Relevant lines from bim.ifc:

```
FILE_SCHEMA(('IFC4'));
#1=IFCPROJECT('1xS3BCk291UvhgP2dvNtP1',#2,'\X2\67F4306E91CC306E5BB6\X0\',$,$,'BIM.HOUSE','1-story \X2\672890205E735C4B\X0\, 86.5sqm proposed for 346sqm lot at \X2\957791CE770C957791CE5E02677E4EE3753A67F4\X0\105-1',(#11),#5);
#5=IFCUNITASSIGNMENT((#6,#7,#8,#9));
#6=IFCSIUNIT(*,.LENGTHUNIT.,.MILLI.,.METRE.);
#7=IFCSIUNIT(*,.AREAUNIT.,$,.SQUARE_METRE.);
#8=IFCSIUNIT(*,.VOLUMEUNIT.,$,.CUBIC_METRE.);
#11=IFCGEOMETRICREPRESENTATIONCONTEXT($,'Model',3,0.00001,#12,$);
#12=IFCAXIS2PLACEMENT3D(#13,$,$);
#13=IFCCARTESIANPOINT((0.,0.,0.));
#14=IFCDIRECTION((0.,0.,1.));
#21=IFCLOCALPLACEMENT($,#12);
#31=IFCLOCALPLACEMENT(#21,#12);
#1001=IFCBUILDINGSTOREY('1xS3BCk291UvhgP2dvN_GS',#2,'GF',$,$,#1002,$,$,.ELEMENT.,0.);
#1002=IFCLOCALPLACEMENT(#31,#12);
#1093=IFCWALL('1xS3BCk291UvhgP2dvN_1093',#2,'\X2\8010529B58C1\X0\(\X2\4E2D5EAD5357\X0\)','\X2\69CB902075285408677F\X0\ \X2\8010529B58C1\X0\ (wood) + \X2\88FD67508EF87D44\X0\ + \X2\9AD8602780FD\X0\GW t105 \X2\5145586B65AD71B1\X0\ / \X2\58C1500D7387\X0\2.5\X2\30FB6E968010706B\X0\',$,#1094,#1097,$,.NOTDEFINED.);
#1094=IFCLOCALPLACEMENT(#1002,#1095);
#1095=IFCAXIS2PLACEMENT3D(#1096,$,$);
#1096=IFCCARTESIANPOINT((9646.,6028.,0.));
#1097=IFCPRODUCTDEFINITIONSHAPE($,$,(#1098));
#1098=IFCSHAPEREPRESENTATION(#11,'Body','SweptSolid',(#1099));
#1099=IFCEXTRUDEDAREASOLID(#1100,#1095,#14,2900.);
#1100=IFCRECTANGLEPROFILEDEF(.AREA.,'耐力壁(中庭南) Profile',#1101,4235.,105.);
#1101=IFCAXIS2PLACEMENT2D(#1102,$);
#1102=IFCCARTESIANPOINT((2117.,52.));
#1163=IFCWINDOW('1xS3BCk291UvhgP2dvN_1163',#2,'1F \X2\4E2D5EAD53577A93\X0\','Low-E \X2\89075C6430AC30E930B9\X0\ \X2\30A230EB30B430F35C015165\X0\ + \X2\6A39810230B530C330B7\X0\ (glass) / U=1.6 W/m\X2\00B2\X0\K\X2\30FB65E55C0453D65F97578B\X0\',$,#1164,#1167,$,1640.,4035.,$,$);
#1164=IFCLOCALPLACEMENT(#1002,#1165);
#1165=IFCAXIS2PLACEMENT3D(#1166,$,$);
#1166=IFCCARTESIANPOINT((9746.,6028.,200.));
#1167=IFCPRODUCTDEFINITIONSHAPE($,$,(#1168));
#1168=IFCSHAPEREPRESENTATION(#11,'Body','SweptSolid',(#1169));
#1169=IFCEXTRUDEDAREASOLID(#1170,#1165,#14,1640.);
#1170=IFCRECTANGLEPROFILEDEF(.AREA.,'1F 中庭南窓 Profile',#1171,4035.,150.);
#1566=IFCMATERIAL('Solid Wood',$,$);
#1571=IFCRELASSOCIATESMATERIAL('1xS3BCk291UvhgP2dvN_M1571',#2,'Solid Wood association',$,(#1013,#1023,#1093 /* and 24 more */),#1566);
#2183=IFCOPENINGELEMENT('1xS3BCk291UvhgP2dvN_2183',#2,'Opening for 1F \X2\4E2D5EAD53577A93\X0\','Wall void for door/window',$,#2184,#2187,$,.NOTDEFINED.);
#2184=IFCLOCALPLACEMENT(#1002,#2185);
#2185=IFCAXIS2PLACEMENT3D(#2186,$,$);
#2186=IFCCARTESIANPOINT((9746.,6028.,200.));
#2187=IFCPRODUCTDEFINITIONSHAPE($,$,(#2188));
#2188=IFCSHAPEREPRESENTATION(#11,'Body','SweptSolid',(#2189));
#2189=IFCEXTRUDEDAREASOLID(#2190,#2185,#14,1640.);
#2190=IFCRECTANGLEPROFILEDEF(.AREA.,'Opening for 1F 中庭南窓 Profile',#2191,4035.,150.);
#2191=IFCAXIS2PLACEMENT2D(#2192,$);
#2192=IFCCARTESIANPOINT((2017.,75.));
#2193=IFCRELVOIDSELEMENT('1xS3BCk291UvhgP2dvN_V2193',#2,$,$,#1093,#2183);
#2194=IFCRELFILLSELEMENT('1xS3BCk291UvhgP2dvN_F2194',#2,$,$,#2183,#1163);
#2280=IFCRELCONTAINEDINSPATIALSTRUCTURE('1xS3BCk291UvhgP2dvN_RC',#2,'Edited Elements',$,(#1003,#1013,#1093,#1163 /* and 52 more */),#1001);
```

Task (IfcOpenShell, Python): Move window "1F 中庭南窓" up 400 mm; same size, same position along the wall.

```python
import numpy as np
import ifcopenshell
import ifcopenshell.api.geometry
import ifcopenshell.util.placement
import ifcopenshell.util.unit

model = ifcopenshell.open("bim.ifc")
unit_scale = ifcopenshell.util.unit.calculate_unit_scale(model)

window = model.by_guid("1xS3BCk291UvhgP2dvN_1163")
opening = window.FillsVoids[0].RelatingOpeningElement
dz = 400.0

shift = np.array([0.0, 0.0, dz])
# The window is not placed relative to its opening, so move both.
for product in (opening, window):
    matrix = ifcopenshell.util.placement.get_local_placement(product.ObjectPlacement)
    matrix[:3, 3] += shift
    ifcopenshell.api.geometry.edit_object_placement(model, product=product, matrix=matrix, is_si=False)

print(f"moved by {dz * unit_scale:+.3f} m")

model.write("bim_updated.ifc")
```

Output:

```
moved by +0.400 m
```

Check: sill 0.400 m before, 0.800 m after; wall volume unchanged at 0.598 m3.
